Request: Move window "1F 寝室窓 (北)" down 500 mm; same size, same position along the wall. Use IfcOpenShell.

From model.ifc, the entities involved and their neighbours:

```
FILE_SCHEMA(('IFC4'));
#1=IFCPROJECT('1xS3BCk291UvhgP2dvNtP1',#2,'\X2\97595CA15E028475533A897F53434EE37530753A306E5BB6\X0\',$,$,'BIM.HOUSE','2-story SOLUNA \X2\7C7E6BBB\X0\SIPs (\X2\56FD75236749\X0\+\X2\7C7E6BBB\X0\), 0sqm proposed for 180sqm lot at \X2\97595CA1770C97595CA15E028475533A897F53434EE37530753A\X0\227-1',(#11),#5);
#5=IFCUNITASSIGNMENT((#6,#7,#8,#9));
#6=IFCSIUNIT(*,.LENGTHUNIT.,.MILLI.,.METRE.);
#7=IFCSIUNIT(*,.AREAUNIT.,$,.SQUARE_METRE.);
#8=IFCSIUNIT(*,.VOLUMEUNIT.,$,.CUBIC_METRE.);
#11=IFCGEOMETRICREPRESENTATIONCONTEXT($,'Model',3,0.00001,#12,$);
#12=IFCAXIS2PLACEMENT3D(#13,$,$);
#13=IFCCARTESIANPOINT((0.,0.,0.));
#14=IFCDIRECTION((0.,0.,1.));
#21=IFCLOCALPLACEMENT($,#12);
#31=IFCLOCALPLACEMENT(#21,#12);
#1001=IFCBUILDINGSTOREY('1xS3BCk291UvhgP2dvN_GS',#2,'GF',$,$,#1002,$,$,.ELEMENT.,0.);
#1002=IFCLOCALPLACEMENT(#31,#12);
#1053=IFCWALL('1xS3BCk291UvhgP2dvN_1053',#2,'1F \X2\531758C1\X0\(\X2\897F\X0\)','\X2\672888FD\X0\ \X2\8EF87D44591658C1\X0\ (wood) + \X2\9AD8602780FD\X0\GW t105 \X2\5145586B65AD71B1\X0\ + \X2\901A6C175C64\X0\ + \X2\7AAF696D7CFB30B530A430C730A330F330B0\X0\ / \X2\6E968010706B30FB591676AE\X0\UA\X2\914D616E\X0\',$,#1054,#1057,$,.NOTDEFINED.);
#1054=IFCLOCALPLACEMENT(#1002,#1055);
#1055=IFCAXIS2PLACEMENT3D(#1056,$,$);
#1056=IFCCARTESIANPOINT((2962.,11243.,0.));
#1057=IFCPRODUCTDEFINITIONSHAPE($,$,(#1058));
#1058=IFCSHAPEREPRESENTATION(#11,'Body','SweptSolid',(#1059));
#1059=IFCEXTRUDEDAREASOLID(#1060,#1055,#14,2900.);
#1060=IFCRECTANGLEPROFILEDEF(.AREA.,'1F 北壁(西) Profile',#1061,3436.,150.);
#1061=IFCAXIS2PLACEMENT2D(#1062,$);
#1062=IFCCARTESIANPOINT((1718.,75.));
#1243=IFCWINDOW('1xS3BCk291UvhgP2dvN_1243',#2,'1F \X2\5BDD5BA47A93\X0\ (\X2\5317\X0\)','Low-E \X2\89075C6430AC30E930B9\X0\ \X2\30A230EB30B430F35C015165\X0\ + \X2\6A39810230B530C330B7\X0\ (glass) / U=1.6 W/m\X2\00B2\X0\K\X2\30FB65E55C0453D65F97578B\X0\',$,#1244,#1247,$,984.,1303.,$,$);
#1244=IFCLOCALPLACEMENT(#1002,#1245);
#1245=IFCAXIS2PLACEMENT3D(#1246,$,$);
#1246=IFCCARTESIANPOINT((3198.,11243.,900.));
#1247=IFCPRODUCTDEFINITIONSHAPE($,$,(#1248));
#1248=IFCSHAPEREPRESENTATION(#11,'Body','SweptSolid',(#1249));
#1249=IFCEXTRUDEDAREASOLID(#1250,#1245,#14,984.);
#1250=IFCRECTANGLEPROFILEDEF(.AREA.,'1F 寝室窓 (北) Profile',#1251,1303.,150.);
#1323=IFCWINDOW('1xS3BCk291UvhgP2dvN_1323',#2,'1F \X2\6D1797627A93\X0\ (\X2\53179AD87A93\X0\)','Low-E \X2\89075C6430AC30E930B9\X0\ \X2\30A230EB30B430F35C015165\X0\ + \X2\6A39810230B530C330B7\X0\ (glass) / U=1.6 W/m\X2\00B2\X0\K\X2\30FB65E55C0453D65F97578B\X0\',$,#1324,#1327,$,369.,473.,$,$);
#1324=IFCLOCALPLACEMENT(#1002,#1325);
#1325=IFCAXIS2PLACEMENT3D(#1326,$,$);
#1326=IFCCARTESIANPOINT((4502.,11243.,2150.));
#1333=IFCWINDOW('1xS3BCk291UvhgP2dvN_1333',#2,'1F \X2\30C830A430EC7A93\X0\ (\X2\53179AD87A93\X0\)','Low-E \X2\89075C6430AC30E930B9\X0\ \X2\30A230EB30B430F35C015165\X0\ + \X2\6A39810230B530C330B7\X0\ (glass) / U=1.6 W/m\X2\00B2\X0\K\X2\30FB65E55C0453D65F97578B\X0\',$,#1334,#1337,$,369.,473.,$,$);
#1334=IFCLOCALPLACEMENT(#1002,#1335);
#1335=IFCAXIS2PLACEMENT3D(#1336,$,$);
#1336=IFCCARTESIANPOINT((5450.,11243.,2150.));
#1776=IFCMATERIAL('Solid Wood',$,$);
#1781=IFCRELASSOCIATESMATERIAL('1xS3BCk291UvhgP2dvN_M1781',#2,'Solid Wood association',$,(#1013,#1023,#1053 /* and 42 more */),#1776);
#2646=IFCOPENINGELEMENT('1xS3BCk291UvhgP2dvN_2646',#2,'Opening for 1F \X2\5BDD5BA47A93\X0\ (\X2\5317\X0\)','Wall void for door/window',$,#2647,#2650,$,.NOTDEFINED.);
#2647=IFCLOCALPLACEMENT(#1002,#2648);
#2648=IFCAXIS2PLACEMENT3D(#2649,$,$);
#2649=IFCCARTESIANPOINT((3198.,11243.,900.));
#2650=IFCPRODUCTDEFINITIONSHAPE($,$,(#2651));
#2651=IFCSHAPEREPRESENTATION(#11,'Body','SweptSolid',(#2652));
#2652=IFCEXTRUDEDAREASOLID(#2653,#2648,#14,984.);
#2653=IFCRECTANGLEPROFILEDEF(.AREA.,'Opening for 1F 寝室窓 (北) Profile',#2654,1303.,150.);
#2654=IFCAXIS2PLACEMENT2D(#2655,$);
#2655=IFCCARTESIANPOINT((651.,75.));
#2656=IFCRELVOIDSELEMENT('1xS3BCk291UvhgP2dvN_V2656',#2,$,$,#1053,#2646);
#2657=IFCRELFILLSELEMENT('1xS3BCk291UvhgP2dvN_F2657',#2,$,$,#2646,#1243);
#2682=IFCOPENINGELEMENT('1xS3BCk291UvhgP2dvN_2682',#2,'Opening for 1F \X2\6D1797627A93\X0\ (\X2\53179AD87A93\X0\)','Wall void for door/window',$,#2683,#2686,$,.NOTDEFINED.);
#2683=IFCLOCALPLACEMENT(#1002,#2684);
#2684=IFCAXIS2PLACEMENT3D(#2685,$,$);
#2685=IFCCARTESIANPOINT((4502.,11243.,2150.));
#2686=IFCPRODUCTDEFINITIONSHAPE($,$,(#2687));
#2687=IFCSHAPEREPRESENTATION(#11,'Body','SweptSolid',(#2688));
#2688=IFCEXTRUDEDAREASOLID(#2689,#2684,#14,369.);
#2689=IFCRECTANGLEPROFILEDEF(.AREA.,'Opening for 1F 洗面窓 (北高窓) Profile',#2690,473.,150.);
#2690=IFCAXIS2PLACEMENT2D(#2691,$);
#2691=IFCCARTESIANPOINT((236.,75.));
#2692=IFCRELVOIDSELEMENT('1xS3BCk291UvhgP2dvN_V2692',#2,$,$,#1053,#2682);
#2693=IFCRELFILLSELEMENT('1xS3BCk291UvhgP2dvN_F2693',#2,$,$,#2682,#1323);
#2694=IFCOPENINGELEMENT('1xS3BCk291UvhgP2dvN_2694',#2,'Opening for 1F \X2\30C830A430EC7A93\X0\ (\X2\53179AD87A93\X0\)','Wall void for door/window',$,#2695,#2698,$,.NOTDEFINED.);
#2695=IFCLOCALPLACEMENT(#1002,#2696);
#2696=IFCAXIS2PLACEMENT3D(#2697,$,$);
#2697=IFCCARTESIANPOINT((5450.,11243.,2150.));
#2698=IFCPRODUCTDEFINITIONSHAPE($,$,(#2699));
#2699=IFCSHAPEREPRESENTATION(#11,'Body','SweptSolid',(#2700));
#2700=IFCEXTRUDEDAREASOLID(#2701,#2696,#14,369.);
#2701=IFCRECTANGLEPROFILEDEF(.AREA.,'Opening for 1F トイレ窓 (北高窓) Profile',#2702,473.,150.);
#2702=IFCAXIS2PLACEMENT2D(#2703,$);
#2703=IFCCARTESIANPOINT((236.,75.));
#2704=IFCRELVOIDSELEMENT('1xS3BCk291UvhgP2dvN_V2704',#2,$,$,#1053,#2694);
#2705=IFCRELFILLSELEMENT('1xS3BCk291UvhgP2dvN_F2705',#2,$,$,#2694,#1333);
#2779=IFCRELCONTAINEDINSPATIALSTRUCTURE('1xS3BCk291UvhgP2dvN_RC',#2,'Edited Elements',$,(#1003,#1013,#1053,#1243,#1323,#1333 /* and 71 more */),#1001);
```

```python
import numpy as np
import ifcopenshell
import ifcopenshell.api.geometry
import ifcopenshell.util.placement
import ifcopenshell.util.unit

model = ifcopenshell.open("model.ifc")
unit_scale = ifcopenshell.util.unit.calculate_unit_scale(model)

window = model.by_id(1243)
opening = window.FillsVoids[0].RelatingOpeningElement
dz = -0.5 / unit_scale

shift = np.array([0.0, 0.0, dz])
# The window is not placed relative to its opening, so move both.
for product in (opening, window):
    matrix = ifcopenshell.util.placement.get_local_placement(product.ObjectPlacement)
    matrix[:3, 3] += shift
    ifcopenshell.api.geometry.edit_object_placement(model, product=product, matrix=matrix, is_si=False)

print(f"moved by {dz * unit_scale:+.3f} m")

model.write("model_updated.ifc")
```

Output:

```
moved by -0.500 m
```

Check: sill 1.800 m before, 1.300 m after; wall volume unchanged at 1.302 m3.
